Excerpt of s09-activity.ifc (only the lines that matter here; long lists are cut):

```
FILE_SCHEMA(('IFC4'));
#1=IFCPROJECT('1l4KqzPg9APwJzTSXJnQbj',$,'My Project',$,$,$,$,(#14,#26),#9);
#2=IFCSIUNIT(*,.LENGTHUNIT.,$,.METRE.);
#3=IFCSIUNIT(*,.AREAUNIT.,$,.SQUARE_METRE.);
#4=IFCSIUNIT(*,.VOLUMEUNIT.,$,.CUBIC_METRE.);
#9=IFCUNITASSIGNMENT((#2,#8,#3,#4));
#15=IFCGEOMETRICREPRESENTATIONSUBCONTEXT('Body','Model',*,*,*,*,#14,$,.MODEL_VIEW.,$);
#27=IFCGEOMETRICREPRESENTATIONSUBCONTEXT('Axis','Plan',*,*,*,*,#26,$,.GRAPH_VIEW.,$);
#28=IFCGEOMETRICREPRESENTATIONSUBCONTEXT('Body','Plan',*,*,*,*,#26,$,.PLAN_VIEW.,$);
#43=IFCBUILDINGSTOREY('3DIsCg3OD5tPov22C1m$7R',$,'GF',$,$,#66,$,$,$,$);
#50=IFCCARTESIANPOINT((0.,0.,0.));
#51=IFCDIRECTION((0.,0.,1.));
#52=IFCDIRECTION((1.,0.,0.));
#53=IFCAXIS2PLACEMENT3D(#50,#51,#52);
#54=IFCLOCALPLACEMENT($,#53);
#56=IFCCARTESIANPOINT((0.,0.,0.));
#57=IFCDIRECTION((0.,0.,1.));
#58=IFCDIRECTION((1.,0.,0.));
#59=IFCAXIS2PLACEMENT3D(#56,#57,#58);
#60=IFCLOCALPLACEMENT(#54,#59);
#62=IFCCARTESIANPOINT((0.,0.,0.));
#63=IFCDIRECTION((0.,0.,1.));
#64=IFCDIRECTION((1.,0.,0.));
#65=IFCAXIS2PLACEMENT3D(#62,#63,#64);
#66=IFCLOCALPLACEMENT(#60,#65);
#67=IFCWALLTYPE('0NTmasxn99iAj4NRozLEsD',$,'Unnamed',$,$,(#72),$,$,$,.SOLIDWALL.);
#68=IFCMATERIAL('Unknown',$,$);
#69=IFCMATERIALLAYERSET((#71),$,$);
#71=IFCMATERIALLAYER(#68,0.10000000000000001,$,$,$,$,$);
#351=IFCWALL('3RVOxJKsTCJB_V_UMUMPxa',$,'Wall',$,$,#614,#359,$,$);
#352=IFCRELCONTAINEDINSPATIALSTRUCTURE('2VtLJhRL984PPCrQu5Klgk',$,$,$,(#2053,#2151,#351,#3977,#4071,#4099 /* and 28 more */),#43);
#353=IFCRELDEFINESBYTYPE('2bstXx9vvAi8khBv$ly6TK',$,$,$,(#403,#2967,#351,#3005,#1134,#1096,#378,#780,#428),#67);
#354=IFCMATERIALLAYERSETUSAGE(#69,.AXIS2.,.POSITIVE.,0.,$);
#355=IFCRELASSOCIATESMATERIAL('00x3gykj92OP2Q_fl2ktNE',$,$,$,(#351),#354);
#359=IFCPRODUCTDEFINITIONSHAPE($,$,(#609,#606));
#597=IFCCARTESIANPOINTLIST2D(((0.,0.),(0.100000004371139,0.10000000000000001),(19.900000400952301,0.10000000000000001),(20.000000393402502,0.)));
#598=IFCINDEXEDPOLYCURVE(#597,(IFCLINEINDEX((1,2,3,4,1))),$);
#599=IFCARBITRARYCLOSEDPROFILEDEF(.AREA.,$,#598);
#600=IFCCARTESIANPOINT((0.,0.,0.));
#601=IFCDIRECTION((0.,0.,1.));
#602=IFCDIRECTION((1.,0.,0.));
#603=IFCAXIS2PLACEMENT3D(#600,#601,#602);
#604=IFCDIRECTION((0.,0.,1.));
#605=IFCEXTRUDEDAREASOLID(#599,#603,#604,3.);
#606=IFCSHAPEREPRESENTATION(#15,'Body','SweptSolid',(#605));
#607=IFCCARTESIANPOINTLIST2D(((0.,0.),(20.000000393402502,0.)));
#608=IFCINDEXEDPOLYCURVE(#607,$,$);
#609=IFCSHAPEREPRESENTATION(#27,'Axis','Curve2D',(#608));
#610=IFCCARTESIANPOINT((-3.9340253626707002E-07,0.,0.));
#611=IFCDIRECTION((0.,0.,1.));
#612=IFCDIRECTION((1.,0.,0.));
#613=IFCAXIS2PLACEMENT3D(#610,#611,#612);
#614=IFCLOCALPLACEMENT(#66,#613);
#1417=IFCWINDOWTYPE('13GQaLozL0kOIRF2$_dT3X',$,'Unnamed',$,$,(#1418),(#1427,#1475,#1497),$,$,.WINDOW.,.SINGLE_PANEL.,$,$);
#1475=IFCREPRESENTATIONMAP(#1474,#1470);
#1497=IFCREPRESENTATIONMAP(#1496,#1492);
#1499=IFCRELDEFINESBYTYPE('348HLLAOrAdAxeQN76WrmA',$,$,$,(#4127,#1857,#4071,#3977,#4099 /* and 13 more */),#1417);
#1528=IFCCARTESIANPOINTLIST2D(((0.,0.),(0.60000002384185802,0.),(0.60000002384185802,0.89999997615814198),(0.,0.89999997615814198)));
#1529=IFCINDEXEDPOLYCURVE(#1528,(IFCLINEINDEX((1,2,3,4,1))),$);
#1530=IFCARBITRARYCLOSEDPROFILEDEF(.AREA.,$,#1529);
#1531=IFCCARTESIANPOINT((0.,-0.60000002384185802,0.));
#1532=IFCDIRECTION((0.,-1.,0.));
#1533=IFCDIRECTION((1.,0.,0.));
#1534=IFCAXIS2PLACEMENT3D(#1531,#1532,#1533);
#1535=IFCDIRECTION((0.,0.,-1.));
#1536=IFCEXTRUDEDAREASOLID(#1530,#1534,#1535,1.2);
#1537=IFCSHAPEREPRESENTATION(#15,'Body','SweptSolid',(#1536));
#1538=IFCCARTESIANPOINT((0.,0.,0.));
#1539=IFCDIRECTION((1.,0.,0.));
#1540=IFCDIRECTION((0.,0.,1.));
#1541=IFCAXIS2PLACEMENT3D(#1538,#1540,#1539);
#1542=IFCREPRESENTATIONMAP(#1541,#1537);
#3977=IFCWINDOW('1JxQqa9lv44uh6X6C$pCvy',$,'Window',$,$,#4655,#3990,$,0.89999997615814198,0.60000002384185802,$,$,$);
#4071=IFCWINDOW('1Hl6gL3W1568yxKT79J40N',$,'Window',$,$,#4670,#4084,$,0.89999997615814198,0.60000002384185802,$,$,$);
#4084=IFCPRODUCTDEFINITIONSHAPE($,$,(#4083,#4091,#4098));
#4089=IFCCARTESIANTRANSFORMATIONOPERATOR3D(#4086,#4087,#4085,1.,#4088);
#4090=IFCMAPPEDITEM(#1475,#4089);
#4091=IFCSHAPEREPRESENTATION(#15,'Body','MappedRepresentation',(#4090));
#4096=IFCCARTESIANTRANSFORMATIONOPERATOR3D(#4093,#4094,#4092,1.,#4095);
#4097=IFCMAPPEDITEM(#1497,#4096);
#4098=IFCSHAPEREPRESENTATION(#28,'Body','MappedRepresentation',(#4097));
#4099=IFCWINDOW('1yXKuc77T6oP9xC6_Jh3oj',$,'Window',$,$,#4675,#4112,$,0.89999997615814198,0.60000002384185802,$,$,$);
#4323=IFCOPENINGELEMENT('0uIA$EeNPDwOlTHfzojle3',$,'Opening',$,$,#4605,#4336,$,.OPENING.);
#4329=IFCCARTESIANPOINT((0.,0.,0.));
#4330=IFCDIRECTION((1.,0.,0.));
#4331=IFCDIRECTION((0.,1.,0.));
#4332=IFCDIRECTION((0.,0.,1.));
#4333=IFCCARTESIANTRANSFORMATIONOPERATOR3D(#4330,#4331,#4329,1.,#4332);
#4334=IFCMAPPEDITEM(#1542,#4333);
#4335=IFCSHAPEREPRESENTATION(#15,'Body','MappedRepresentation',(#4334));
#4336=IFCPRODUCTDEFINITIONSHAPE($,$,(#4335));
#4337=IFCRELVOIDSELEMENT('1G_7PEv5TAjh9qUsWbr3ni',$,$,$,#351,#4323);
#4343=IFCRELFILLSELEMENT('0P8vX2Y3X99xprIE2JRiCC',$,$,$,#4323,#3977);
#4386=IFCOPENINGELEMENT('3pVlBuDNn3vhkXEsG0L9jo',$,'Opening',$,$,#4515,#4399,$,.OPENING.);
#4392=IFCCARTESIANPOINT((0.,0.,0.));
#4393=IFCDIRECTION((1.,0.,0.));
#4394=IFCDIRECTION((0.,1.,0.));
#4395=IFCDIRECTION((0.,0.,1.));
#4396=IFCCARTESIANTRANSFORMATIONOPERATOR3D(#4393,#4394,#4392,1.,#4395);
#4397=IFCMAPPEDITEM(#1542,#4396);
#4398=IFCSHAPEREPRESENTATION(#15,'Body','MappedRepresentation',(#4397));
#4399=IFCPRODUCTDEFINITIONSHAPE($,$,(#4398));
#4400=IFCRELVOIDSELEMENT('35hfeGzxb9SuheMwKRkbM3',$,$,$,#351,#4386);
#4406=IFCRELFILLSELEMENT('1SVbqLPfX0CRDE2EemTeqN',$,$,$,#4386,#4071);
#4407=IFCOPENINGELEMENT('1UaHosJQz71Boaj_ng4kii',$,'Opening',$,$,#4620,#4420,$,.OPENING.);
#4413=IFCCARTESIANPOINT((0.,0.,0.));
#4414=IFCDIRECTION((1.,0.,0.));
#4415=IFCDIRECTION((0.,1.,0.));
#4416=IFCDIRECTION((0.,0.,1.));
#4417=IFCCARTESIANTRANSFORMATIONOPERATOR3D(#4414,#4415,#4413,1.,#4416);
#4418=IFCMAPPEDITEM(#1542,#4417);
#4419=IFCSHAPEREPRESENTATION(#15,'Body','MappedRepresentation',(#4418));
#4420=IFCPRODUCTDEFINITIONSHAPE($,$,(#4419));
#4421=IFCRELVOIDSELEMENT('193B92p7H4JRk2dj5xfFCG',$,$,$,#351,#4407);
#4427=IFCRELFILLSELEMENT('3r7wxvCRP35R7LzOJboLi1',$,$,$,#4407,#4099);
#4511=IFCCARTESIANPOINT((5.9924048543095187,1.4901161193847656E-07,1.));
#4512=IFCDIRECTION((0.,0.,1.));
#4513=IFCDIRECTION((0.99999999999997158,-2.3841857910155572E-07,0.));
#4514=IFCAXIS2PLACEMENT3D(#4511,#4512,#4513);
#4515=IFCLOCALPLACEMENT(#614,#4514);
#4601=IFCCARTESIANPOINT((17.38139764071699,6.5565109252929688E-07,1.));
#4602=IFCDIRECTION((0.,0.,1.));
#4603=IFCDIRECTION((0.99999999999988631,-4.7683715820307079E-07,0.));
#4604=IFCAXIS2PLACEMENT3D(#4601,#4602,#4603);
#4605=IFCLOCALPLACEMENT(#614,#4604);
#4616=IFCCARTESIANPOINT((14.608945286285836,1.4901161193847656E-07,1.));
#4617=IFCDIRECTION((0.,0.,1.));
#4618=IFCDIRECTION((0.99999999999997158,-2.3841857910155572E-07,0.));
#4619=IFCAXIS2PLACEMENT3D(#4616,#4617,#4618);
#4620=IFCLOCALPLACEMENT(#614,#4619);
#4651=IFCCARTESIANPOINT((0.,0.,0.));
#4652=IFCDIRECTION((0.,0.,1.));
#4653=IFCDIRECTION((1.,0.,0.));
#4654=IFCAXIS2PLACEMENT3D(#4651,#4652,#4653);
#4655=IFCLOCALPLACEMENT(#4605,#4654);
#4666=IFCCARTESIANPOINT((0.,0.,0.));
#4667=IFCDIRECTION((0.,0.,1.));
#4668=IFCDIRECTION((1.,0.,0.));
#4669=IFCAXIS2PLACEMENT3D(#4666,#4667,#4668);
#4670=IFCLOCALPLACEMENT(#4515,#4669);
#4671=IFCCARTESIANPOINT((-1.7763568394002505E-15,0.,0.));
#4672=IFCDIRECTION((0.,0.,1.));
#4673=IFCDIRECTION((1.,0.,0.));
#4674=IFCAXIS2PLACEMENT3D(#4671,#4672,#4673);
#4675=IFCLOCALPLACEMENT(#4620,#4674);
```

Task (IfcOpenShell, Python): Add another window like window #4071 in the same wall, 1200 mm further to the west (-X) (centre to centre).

```python
import ifcopenshell
import ifcopenshell.api.feature
import ifcopenshell.api.geometry
import ifcopenshell.api.root
import ifcopenshell.geom
import ifcopenshell.util.element
import ifcopenshell.util.placement
import ifcopenshell.util.shape
import ifcopenshell.util.unit

model = ifcopenshell.open("s09-activity.ifc")
unit_scale = ifcopenshell.util.unit.calculate_unit_scale(model)
settings = ifcopenshell.geom.settings()


def volume(element):
    """Net volume in cubic metres, openings subtracted."""
    shape = ifcopenshell.geom.create_shape(settings, element)
    return ifcopenshell.util.shape.get_volume(shape.geometry)


window = model.by_guid("1Hl6gL3W1568yxKT79J40N")
opening = window.FillsVoids[0].RelatingOpeningElement
wall = opening.VoidsElements[0].RelatingBuildingElement
before = volume(wall)
shift = ifcopenshell.util.placement.get_local_placement(wall.ObjectPlacement)[:3, 0] * -1.2 / unit_scale

# copy_class copies the void relationship, type, container and properties, but no geometry.
new_opening = ifcopenshell.api.root.copy_class(model, product=opening)
new_opening.Representation = ifcopenshell.util.element.copy_deep(
    model, opening.Representation, exclude=["IfcGeometricRepresentationContext", "IfcRepresentationMap"]
)
new_window = ifcopenshell.api.root.copy_class(model, product=window)
new_window.Representation = ifcopenshell.util.element.copy_deep(
    model, window.Representation, exclude=["IfcGeometricRepresentationContext", "IfcRepresentationMap"]
)
ifcopenshell.api.feature.add_filling(model, opening=new_opening, element=new_window)

for old, new in ((opening, new_opening), (window, new_window)):
    matrix = ifcopenshell.util.placement.get_local_placement(old.ObjectPlacement)
    matrix[:3, 3] += shift
    ifcopenshell.api.geometry.edit_object_placement(model, product=new, matrix=matrix, is_si=False)

after = volume(wall)

print(f"wall volume {before:.3f} -> {after:.3f} m3")

model.write("s09-activity_rev.ifc")
```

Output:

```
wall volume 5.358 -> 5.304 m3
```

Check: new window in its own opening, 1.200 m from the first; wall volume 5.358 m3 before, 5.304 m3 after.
